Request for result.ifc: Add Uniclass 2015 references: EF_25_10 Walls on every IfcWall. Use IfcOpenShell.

First a look at what the model holds.

```python
import ifcopenshell

model = ifcopenshell.open("result.ifc")
print(model.schema)
print("classifications:", [c.Name for c in model.by_type("IfcClassification")])
for ifc_class in ("IfcDoor", "IfcRoof", "IfcStair", "IfcWall", "IfcWindow"):
    print(ifc_class, len(model.by_type(ifc_class)))
```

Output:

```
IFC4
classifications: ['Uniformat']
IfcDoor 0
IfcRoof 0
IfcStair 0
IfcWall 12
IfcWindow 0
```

```python
import ifcopenshell
import ifcopenshell.api.classification

model = ifcopenshell.open("result.ifc")

system = ifcopenshell.api.classification.add_classification(model, classification="Uniclass 2015")

codes = {
    "IfcWall": ("EF_25_10", "Walls"),
}
for ifc_class, (code, name) in codes.items():
    products = model.by_type(ifc_class)
    ifcopenshell.api.classification.add_reference(
        model, products=products, classification=system, identification=code, name=name
    )
    print(code, len(products))

model.write("result_edited.ifc")
```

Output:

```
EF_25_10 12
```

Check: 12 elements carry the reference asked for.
